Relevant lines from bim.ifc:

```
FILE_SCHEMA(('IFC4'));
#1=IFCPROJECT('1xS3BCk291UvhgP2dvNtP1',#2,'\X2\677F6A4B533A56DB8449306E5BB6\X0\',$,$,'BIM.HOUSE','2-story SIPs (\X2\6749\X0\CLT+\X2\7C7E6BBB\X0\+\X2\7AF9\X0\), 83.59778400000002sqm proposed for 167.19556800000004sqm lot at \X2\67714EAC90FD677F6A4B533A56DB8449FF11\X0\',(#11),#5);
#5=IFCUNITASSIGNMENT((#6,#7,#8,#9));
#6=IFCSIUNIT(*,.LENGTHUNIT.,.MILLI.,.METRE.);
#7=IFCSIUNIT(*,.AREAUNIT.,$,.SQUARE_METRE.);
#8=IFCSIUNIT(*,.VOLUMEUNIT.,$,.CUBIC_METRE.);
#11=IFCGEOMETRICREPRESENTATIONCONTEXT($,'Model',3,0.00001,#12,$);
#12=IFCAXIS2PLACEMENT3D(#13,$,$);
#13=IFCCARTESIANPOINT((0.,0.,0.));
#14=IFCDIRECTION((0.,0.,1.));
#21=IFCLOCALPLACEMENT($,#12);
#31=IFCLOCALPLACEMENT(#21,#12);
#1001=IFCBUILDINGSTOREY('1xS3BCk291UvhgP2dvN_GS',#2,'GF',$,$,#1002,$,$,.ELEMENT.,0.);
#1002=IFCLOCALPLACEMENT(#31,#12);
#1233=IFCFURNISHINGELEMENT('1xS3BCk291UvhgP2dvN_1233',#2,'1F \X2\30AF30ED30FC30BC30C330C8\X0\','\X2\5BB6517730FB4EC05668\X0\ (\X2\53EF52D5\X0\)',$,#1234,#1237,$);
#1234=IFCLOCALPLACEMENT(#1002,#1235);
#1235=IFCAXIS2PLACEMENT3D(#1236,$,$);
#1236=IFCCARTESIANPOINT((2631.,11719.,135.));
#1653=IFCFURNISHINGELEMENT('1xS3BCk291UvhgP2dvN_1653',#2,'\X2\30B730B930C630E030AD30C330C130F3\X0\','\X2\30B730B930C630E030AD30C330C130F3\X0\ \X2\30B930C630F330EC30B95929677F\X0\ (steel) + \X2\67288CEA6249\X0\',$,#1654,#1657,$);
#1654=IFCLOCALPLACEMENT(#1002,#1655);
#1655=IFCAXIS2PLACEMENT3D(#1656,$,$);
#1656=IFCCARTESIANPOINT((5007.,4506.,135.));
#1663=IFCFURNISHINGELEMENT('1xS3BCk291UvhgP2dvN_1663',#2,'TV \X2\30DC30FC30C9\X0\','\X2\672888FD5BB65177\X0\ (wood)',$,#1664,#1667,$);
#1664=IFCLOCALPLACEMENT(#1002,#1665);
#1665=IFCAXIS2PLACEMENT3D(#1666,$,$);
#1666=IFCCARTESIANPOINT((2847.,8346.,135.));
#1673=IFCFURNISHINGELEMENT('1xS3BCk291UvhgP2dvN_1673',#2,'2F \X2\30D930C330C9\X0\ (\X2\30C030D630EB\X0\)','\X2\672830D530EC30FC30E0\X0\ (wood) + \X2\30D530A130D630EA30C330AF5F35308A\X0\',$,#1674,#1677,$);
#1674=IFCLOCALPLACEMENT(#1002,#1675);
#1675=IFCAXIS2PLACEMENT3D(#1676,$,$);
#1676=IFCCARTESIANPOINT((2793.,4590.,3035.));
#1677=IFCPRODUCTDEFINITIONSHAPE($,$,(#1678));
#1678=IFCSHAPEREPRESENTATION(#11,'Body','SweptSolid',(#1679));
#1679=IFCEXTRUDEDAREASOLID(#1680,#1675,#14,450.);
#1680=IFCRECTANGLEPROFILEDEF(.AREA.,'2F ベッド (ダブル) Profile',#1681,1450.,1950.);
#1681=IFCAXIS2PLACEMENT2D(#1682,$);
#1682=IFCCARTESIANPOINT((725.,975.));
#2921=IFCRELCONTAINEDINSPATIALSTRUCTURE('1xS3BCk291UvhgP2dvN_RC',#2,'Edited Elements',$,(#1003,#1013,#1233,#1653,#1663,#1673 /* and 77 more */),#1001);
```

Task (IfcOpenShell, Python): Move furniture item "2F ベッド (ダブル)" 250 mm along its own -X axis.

```python
import ifcopenshell
import ifcopenshell.api.geometry
import ifcopenshell.util.placement
import ifcopenshell.util.unit

model = ifcopenshell.open("bim.ifc")
unit_scale = ifcopenshell.util.unit.calculate_unit_scale(model)

item = model.by_guid("1xS3BCk291UvhgP2dvN_1673")
matrix = ifcopenshell.util.placement.get_local_placement(item.ObjectPlacement)
matrix[:3, 3] -= matrix[:3, 0] * 0.25 / unit_scale
ifcopenshell.api.geometry.edit_object_placement(model, product=item, matrix=matrix, is_si=False)

print(ifcopenshell.util.placement.get_local_placement(item.ObjectPlacement).round(3) + 0.0)

model.write("bim_v2.ifc")
```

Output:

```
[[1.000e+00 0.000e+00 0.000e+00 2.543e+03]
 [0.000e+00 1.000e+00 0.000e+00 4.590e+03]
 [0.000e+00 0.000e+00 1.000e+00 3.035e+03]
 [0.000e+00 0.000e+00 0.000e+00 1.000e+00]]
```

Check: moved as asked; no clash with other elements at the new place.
